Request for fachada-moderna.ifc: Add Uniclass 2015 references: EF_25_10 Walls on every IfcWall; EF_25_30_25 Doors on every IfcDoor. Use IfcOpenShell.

First a look at what the model holds.

```python
import ifcopenshell

model = ifcopenshell.open("fachada-moderna.ifc")
print(model.schema)
print("classifications:", [c.Name for c in model.by_type("IfcClassification")])
for ifc_class in ("IfcDoor", "IfcRoof", "IfcStair", "IfcWall", "IfcWindow"):
    print(ifc_class, len(model.by_type(ifc_class)))
```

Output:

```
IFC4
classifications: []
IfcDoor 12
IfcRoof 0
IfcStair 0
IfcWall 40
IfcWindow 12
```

```python
import ifcopenshell
import ifcopenshell.api.classification

model = ifcopenshell.open("fachada-moderna.ifc")

system = ifcopenshell.api.classification.add_classification(model, classification="Uniclass 2015")

codes = {
    "IfcWall": ("EF_25_10", "Walls"),
    "IfcDoor": ("EF_25_30_25", "Doors"),
}
for ifc_class, (code, name) in codes.items():
    products = model.by_type(ifc_class)
    ifcopenshell.api.classification.add_reference(
        model, products=products, classification=system, identification=code, name=name
    )
    print(code, len(products))

model.write("fachada-moderna-out.ifc")
```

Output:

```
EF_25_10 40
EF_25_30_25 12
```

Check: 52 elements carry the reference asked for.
